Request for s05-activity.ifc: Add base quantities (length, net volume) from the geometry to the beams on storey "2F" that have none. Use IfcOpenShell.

First a look at what the model holds.

```python
import ifcopenshell
import ifcopenshell.util.element
import ifcopenshell.util.unit

model = ifcopenshell.open("s05-activity.ifc")
print(model.schema)
for unit_type in ("LENGTHUNIT", "AREAUNIT", "VOLUMEUNIT"):
    print(unit_type, ifcopenshell.util.unit.calculate_unit_scale(model, unit_type))
storey = next(s for s in model.by_type("IfcBuildingStorey") if s.Name == "2F")
beams = [e for e in ifcopenshell.util.element.get_decomposition(storey) if e.is_a("IfcBeam")]
for e in sorted(beams, key=lambda e: e.id()):
    print(e.id(), e.is_a(), e.Name, list(ifcopenshell.util.element.get_psets(e, qtos_only=True)), sep=" | ")
```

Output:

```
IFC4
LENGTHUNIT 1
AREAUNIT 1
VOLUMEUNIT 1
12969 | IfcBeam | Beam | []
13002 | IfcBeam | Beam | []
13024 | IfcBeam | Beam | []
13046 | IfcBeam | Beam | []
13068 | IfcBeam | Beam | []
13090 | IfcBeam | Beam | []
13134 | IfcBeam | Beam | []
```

```python
import ifcopenshell
import ifcopenshell.api.pset
import ifcopenshell.geom
import ifcopenshell.util.element
import ifcopenshell.util.shape
import ifcopenshell.util.unit

model = ifcopenshell.open("s05-activity.ifc")
unit_scale = ifcopenshell.util.unit.calculate_unit_scale(model)
volume_scale = ifcopenshell.util.unit.calculate_unit_scale(model, "VOLUMEUNIT")
settings = ifcopenshell.geom.settings()

storey = next(s for s in model.by_type("IfcBuildingStorey") if s.Name == "2F")
beams = [e for e in ifcopenshell.util.element.get_decomposition(storey) if e.is_a("IfcBeam")]

for e in sorted(beams, key=lambda e: e.id()):
    if ifcopenshell.util.element.get_psets(e, qtos_only=True, should_inherit=False):
        continue
    # Geometry comes back in metres, in the element's own axes.
    shape = ifcopenshell.geom.create_shape(settings, e)
    values = {
        "Length": ifcopenshell.util.shape.get_max_xyz(shape.geometry) / unit_scale,
        "NetVolume": ifcopenshell.util.shape.get_volume(shape.geometry) / volume_scale,
    }
    qto = ifcopenshell.api.pset.add_qto(model, product=e, name="Qto_BeamBaseQuantities")
    ifcopenshell.api.pset.edit_qto(model, qto=qto, properties=values)
    print(e.id(), {k: round(v, 3) for k, v in values.items()})

model.write("s05-activity_updated.ifc")
```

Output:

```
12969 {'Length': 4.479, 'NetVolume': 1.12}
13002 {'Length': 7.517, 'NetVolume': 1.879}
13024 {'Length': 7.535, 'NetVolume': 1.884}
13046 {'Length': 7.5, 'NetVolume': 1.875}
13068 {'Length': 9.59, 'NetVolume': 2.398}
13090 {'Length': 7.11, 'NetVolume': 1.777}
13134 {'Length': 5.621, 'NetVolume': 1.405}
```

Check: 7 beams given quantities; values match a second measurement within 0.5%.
